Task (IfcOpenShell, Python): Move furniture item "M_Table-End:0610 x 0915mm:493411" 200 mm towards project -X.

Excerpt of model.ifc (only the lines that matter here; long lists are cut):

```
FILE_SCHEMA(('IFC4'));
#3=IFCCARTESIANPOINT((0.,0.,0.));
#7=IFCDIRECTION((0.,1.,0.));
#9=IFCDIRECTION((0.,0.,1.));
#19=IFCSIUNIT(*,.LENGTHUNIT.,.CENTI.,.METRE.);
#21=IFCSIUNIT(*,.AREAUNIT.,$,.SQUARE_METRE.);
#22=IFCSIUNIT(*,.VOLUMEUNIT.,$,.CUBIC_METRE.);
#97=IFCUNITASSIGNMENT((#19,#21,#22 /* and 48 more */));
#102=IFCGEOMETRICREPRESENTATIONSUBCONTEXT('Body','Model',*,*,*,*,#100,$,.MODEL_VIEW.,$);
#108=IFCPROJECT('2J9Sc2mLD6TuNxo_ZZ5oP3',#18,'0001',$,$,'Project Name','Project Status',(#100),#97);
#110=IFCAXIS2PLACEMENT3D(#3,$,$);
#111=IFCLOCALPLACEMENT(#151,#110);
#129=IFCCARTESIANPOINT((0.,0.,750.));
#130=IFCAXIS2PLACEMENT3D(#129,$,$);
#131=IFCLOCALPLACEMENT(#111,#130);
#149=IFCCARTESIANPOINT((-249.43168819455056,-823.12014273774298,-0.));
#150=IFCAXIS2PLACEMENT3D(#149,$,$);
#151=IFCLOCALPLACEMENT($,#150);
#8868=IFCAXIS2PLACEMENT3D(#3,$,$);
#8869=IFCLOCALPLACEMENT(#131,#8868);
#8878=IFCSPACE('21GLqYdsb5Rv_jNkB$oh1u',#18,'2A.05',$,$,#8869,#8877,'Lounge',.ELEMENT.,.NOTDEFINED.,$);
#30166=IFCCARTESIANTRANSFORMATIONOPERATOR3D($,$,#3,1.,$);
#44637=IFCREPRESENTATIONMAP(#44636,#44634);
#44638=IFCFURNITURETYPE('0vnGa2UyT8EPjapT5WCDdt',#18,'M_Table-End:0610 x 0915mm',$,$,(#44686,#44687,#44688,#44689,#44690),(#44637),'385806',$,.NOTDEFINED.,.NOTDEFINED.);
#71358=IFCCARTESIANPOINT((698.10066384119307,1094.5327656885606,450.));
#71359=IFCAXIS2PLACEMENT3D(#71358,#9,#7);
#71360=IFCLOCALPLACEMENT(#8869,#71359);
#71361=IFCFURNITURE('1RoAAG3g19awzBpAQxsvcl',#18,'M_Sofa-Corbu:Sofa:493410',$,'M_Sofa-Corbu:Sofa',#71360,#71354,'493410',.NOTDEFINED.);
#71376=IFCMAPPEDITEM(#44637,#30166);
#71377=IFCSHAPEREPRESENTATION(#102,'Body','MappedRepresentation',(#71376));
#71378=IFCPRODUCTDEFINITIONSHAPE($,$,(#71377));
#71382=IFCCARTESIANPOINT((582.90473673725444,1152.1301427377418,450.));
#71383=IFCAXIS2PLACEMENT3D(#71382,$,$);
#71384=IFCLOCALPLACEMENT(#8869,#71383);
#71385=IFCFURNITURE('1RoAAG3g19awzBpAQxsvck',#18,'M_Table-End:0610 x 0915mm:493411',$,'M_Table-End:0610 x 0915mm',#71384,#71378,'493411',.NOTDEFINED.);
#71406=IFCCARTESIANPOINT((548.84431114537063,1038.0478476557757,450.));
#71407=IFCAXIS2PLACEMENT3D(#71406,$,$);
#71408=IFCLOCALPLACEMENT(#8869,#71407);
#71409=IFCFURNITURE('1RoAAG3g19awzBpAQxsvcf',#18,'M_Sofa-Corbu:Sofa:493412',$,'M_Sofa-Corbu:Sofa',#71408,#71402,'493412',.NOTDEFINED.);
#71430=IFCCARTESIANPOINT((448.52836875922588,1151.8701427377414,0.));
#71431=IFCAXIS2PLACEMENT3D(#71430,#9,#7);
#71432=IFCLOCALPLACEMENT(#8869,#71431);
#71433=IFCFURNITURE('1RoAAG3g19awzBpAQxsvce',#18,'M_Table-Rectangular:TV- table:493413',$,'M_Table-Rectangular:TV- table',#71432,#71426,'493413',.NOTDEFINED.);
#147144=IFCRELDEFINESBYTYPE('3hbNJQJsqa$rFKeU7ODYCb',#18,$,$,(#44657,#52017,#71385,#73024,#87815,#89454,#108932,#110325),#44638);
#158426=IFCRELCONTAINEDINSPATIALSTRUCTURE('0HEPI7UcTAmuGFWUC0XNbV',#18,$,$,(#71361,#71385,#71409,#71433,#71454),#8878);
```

```python
import ifcopenshell
import ifcopenshell.api.geometry
import ifcopenshell.util.placement
import ifcopenshell.util.unit

model = ifcopenshell.open("model.ifc")
unit_scale = ifcopenshell.util.unit.calculate_unit_scale(model)

item = model.by_id(71385)
matrix = ifcopenshell.util.placement.get_local_placement(item.ObjectPlacement)
matrix[0, 3] -= 0.2 / unit_scale
ifcopenshell.api.geometry.edit_object_placement(model, product=item, matrix=matrix, is_si=False)

print(ifcopenshell.util.placement.get_local_placement(item.ObjectPlacement).round(3) + 0.0)

model.write("model-out.ifc")
```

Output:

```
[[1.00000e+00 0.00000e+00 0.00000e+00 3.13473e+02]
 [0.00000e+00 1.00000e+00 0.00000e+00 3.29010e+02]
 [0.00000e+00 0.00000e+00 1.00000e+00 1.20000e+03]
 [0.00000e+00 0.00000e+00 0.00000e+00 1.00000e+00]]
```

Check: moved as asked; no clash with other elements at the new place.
